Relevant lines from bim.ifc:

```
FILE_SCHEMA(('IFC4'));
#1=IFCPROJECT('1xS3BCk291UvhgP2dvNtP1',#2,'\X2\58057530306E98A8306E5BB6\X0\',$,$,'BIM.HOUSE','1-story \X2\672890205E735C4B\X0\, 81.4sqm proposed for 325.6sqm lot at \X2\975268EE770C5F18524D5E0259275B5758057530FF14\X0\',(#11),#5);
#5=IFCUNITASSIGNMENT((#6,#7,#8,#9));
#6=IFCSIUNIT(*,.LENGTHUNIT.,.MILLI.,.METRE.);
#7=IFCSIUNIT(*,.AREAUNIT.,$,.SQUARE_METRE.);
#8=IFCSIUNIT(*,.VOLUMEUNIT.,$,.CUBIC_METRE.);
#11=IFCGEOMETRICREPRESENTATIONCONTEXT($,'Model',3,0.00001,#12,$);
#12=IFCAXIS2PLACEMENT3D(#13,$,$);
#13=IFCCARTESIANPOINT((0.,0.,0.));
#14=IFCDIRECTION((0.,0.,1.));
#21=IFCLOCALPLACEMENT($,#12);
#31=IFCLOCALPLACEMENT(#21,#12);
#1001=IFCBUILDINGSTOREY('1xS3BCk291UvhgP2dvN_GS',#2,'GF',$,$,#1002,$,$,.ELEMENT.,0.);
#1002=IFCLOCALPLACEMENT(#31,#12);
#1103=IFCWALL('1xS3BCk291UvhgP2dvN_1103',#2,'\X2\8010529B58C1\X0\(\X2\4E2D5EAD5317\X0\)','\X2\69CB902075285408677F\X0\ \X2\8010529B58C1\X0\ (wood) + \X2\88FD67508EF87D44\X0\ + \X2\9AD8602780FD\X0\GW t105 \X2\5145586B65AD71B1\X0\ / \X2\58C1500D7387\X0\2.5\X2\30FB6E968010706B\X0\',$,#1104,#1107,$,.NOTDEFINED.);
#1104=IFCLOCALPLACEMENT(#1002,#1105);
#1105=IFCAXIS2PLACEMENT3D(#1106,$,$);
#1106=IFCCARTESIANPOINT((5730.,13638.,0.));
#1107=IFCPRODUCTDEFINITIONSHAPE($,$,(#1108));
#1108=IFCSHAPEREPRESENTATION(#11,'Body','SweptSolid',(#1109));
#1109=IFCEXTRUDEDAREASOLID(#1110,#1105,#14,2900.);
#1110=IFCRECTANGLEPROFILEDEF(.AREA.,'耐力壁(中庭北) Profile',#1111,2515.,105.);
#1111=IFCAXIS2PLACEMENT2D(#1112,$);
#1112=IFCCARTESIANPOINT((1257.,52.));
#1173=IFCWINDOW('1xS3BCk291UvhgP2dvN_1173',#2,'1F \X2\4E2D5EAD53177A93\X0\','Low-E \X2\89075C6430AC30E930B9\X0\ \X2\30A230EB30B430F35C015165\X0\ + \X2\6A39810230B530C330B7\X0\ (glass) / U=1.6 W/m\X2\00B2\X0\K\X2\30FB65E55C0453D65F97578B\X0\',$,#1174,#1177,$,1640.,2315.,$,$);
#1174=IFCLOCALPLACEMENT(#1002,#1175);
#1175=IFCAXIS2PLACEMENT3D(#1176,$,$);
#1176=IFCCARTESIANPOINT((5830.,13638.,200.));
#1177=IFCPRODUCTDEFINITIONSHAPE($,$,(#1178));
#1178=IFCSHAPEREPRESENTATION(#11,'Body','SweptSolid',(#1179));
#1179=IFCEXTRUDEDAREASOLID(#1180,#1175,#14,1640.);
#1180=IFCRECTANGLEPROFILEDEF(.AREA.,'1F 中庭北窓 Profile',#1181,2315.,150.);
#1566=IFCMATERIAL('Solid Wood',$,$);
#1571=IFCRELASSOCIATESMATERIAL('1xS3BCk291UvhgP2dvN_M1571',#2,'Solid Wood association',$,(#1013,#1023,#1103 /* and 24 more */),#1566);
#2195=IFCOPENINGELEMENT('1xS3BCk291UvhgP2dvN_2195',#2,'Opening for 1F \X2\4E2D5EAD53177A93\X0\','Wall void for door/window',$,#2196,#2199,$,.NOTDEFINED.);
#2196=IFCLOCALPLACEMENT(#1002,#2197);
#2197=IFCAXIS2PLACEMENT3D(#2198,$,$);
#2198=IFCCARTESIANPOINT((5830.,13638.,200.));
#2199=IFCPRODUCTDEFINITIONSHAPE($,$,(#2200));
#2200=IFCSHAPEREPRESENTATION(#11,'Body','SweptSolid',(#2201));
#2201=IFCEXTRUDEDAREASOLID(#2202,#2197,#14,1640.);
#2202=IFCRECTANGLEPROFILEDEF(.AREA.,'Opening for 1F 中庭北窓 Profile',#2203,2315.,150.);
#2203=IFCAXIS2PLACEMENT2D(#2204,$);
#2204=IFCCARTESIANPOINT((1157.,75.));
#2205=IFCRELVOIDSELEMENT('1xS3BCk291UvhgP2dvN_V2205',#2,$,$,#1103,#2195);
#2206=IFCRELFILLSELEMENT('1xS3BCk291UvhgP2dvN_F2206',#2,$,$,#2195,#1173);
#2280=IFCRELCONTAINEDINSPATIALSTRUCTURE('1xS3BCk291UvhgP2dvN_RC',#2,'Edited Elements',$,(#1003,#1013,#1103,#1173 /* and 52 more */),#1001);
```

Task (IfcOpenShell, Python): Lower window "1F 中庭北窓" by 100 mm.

```python
import numpy as np
import ifcopenshell
import ifcopenshell.api.geometry
import ifcopenshell.util.placement
import ifcopenshell.util.unit

model = ifcopenshell.open("bim.ifc")
unit_scale = ifcopenshell.util.unit.calculate_unit_scale(model)

window = model.by_id(1173)
opening = window.FillsVoids[0].RelatingOpeningElement
dz = -0.1 / unit_scale

shift = np.array([0.0, 0.0, dz])
# The window is not placed relative to its opening, so move both.
for product in (opening, window):
    matrix = ifcopenshell.util.placement.get_local_placement(product.ObjectPlacement)
    matrix[:3, 3] += shift
    ifcopenshell.api.geometry.edit_object_placement(model, product=product, matrix=matrix, is_si=False)

print(f"moved by {dz * unit_scale:+.3f} m")

model.write("bim_updated.ifc")
```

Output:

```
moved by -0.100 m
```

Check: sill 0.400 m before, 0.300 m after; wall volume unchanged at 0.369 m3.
